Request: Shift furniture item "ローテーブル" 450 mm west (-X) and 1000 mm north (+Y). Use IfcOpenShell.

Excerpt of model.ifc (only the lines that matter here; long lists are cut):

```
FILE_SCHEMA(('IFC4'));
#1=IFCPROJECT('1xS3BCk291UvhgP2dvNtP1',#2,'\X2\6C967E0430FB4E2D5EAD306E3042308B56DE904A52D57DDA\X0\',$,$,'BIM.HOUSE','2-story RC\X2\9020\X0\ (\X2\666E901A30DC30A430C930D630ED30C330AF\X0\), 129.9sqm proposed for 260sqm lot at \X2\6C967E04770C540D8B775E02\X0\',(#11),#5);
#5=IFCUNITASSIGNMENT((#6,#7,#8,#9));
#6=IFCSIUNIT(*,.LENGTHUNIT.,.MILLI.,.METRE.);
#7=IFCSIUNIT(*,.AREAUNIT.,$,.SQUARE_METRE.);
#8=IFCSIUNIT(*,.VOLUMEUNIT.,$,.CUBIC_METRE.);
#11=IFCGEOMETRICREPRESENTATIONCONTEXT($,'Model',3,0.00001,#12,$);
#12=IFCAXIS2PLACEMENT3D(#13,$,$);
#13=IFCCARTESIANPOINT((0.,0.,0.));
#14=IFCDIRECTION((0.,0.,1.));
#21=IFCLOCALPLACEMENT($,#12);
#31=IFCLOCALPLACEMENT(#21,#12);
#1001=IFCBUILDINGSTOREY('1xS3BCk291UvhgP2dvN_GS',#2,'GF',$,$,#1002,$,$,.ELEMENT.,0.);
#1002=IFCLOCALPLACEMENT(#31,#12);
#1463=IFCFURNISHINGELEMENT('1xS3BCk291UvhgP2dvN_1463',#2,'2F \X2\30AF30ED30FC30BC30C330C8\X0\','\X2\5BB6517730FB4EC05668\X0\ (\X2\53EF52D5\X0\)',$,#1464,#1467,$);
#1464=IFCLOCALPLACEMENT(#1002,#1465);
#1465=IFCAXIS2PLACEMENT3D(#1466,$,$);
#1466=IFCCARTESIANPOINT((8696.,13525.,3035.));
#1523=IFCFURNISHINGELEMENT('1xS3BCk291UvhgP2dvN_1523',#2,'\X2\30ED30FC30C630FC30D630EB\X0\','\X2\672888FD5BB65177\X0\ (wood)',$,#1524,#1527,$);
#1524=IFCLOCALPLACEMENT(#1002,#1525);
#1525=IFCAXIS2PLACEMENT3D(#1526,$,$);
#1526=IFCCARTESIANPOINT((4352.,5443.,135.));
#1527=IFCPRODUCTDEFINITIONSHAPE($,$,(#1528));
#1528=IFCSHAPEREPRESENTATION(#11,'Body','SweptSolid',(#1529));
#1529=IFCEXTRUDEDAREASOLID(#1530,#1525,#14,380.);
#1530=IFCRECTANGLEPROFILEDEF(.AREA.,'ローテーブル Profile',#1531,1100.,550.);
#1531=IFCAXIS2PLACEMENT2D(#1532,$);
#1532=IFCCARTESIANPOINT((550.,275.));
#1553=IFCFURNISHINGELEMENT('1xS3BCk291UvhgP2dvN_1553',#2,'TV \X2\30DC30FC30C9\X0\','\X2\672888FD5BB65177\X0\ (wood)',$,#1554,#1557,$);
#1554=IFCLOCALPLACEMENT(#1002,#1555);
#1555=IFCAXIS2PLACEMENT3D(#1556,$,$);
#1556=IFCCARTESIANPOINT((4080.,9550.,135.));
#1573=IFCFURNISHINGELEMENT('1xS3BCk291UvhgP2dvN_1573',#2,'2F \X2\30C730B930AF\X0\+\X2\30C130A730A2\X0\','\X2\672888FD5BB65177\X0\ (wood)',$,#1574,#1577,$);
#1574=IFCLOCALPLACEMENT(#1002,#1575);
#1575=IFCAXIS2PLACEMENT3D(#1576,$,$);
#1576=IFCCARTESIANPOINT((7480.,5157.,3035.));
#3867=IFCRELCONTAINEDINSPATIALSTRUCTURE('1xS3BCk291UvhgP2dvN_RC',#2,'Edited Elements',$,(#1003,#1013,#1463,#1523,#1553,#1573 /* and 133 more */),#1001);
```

```python
import ifcopenshell
import ifcopenshell.api.geometry
import ifcopenshell.util.placement

model = ifcopenshell.open("model.ifc")

item = model.by_guid("1xS3BCk291UvhgP2dvN_1523")
matrix = ifcopenshell.util.placement.get_local_placement(item.ObjectPlacement)
matrix[0, 3] -= 450.0
matrix[1, 3] += 1000.0
ifcopenshell.api.geometry.edit_object_placement(model, product=item, matrix=matrix, is_si=False)

print(ifcopenshell.util.placement.get_local_placement(item.ObjectPlacement).round(3) + 0.0)

model.write("model_v2.ifc")
```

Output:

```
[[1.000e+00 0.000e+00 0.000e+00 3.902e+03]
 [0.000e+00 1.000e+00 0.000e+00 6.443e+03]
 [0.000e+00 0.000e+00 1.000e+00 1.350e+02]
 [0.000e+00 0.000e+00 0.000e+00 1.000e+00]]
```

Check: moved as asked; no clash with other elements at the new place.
